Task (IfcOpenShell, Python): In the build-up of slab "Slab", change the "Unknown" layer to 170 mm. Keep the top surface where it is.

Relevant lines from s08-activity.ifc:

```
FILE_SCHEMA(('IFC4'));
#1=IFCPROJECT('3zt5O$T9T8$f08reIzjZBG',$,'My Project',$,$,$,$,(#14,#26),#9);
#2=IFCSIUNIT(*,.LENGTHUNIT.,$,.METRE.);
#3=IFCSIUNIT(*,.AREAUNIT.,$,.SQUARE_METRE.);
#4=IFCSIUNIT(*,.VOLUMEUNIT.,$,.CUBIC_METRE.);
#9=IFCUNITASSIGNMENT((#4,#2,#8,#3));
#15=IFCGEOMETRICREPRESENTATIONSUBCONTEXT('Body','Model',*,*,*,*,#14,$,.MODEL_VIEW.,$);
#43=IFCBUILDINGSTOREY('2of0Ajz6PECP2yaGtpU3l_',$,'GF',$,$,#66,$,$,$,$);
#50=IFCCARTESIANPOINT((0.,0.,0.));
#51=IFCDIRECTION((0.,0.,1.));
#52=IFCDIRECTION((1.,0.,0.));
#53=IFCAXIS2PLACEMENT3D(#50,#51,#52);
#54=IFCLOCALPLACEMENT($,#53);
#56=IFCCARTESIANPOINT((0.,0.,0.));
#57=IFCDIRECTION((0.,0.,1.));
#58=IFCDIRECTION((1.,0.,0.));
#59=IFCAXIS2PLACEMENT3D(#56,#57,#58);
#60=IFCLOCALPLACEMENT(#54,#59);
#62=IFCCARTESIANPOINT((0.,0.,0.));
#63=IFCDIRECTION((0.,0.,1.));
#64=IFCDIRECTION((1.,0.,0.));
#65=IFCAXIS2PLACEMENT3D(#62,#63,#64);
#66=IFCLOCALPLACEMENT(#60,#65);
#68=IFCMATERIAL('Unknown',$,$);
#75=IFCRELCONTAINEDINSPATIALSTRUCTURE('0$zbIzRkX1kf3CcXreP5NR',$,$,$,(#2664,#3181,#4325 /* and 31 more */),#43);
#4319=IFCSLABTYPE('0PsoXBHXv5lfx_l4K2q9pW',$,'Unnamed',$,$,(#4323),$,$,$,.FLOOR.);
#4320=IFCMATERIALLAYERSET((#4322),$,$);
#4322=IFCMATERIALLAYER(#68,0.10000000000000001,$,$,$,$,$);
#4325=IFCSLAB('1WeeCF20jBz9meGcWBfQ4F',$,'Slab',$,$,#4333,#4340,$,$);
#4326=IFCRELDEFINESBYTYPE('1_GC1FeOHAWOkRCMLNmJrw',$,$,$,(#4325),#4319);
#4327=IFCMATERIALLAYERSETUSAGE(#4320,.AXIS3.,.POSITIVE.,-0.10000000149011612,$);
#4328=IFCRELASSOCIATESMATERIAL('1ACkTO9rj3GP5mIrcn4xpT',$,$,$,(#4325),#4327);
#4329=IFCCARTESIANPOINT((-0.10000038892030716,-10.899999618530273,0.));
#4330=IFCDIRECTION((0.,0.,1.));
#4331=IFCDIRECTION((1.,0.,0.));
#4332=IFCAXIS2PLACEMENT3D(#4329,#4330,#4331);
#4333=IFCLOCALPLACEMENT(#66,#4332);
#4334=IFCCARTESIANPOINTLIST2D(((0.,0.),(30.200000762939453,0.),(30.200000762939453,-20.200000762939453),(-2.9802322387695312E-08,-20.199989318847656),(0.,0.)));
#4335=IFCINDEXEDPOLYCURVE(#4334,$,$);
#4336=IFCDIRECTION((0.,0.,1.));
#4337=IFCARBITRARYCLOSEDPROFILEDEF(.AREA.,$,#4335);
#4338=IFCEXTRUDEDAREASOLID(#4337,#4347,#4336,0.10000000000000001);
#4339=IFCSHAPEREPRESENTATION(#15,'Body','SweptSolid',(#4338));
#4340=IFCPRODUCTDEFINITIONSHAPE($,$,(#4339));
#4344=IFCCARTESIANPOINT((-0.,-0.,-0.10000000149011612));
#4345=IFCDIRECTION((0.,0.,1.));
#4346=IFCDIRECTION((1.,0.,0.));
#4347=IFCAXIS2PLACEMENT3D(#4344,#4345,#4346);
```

```python
import ifcopenshell
import ifcopenshell.util.element
import ifcopenshell.util.representation
import ifcopenshell.util.unit

model = ifcopenshell.open("s08-activity.ifc")
unit_scale = ifcopenshell.util.unit.calculate_unit_scale(model)

layer_set = model.by_id(4320)
layer = next(l for l in layer_set.MaterialLayers if l.Material and l.Material.Name == "Unknown")
change = 0.17 / unit_scale - layer.LayerThickness
layer.LayerThickness += change

# Geometry does not follow the layer set by itself.
slabs = [e for e in ifcopenshell.util.element.get_elements_by_material(model, layer_set) if e.is_a("IfcSlab")]
for slab in sorted(slabs, key=lambda e: e.id()):
    body = ifcopenshell.util.representation.get_representation(slab, "Model", "Body")
    solid = body.Items[0]
    old_depth = solid.Depth
    solid.Depth += change
    # Extruded upwards: lower the start of the extrusion so the top stays.
    x, y, z = solid.Position.Location.Coordinates
    solid.Position.Location = model.createIfcCartesianPoint((x, y, z - change))
    print(slab.id(), f"{old_depth:g} -> {solid.Depth:g}")

# The layers are counted up from the underside, which has moved.
for usage in {ifcopenshell.util.element.get_material(slab) for slab in slabs}:
    usage.OffsetFromReferenceLine -= change

model.write("s08-activity_updated.ifc")
```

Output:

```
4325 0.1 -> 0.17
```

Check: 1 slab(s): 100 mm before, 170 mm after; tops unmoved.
